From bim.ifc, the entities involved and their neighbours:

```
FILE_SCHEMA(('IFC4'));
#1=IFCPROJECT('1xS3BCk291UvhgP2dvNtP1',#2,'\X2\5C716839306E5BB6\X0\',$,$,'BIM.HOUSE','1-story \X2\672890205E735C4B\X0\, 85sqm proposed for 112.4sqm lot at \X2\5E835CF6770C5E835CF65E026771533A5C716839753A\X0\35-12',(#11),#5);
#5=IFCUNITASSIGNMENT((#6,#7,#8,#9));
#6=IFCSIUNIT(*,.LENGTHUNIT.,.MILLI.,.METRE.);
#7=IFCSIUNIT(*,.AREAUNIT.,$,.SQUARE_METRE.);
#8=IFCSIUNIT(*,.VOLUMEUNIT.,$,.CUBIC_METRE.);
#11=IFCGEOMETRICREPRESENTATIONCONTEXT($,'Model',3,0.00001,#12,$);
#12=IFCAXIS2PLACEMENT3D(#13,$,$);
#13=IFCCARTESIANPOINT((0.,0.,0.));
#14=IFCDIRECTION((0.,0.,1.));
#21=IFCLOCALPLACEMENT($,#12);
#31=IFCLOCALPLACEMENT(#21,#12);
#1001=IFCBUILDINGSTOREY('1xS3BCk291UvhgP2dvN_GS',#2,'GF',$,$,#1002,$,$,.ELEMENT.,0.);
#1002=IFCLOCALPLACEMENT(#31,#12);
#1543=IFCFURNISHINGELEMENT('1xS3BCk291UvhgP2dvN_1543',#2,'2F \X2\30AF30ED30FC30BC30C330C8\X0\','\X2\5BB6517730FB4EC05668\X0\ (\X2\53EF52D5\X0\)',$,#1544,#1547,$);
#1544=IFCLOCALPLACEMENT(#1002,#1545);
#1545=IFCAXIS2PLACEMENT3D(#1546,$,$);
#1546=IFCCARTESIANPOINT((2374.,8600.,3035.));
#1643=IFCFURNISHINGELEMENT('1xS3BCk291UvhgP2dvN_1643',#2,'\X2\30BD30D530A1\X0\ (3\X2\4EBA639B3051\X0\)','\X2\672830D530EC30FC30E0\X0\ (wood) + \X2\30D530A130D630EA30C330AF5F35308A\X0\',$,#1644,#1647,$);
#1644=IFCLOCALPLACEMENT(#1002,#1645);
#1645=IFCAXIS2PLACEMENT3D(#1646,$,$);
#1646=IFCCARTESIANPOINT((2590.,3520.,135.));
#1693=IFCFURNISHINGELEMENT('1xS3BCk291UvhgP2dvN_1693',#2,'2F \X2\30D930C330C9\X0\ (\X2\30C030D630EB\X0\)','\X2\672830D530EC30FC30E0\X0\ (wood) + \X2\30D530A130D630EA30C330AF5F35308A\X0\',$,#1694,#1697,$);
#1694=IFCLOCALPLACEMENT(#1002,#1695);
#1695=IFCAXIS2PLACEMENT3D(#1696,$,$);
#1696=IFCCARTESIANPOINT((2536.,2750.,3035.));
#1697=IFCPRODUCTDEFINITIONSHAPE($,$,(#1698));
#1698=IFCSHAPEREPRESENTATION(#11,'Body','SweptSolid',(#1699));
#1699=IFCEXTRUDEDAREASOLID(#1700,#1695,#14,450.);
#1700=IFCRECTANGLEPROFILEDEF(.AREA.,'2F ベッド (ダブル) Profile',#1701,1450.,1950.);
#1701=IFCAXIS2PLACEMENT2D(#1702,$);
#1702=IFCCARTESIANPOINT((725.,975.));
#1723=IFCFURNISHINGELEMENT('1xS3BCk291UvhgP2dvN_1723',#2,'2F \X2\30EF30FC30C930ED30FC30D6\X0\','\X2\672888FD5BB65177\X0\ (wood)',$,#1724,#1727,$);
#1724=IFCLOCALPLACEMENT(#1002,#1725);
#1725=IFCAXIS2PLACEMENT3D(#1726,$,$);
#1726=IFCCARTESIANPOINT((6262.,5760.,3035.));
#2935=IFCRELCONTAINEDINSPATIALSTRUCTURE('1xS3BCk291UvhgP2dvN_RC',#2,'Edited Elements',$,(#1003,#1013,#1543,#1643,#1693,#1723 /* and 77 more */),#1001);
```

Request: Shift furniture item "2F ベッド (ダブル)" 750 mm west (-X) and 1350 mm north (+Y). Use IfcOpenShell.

```python
import ifcopenshell
import ifcopenshell.api.geometry
import ifcopenshell.util.placement

model = ifcopenshell.open("bim.ifc")

item = model.by_guid("1xS3BCk291UvhgP2dvN_1693")
matrix = ifcopenshell.util.placement.get_local_placement(item.ObjectPlacement)
matrix[0, 3] -= 750.0
matrix[1, 3] += 1350.0
ifcopenshell.api.geometry.edit_object_placement(model, product=item, matrix=matrix, is_si=False)

print(ifcopenshell.util.placement.get_local_placement(item.ObjectPlacement).round(3) + 0.0)

model.write("bim_edited.ifc")
```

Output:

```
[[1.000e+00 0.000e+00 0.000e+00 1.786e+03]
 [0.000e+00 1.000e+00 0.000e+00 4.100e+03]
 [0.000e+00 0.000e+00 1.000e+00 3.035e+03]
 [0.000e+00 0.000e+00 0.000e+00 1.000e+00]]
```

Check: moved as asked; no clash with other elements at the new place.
